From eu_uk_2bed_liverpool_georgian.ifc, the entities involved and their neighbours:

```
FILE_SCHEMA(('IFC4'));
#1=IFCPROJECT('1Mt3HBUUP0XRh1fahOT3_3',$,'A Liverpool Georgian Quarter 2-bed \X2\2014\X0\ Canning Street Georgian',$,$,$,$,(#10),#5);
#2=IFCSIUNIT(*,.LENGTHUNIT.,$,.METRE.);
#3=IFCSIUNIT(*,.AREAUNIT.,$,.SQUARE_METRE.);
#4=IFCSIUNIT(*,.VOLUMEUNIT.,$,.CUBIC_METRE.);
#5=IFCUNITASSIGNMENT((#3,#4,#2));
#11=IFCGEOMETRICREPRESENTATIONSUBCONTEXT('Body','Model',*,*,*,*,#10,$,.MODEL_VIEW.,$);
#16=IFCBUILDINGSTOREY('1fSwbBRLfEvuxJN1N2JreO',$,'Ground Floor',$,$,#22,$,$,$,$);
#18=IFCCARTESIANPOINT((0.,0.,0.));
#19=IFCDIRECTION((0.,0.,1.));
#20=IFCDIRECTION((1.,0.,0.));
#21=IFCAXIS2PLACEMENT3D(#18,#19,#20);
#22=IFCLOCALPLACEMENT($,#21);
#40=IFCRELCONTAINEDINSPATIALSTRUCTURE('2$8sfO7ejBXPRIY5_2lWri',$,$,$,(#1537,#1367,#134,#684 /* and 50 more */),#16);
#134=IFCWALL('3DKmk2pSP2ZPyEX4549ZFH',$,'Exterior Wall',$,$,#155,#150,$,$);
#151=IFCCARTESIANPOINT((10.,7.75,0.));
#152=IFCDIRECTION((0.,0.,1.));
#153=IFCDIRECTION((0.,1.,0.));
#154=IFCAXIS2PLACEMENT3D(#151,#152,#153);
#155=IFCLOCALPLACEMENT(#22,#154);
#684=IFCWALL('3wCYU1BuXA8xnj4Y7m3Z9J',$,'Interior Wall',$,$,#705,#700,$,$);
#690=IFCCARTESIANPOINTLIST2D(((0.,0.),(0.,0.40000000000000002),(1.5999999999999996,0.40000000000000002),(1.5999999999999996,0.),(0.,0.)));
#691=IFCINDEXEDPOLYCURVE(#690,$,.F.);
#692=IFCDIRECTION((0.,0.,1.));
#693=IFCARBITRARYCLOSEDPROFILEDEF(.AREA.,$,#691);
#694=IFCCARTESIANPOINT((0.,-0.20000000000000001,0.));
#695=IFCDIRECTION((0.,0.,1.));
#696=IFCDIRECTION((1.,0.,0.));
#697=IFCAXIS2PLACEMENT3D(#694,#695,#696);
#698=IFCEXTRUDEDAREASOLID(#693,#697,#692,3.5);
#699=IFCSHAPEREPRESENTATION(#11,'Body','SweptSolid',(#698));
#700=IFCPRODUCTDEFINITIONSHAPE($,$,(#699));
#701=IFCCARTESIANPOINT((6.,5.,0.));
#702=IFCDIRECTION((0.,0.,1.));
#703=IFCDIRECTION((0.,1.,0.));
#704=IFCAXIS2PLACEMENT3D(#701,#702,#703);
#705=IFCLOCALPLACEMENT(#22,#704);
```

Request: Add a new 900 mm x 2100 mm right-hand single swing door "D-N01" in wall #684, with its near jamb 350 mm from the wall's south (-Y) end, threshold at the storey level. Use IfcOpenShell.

```python
import numpy as np
import ifcopenshell
import ifcopenshell.api.feature
import ifcopenshell.api.geometry
import ifcopenshell.api.root
import ifcopenshell.api.spatial
import ifcopenshell.geom
import ifcopenshell.util.element
import ifcopenshell.util.placement
import ifcopenshell.util.representation
import ifcopenshell.util.shape
import ifcopenshell.util.unit

model = ifcopenshell.open("eu_uk_2bed_liverpool_georgian.ifc")
unit_scale = ifcopenshell.util.unit.calculate_unit_scale(model)
settings = ifcopenshell.geom.settings()


def volume(element):
    """Net volume in cubic metres, openings subtracted."""
    shape = ifcopenshell.geom.create_shape(settings, element)
    return ifcopenshell.util.shape.get_volume(shape.geometry)


wall = model.by_id(684)
storey = ifcopenshell.util.element.get_container(wall, ifc_class="IfcBuildingStorey")
context = ifcopenshell.util.representation.get_context(model, "Model", "Body", "MODEL_VIEW")
before = volume(wall)

width, height, from_end, sill = 0.9, 2.1, 0.35, 0.0  # metres

# The wall runs along its own X axis, and the end named is its -X end.
wall_shape = ifcopenshell.geom.create_shape(settings, wall)
x, y, z = ifcopenshell.util.shape.get_vertices(wall_shape.geometry).T
start = x.min() + from_end
face, thickness = float(y.min()), float(y.max() - y.min())
wall_matrix = ifcopenshell.util.placement.get_local_placement(wall.ObjectPlacement)
level = ifcopenshell.util.placement.get_local_placement(storey.ObjectPlacement)[2, 3]


def in_wall(x, y):
    """Placement at x, y metres in the wall's axes, at sill height."""
    matrix = wall_matrix.copy()
    matrix[:, 3] = wall_matrix @ np.array([x / unit_scale, y / unit_scale, 0.0, 1.0])
    matrix[2, 3] = level + sill / unit_scale
    return matrix


# Opening: a box that overshoots both wall faces by 50 mm.
opening = ifcopenshell.api.root.create_entity(model, ifc_class="IfcOpeningElement", predefined_type="OPENING")
box = ifcopenshell.api.geometry.add_wall_representation(
    model, context=context, length=width, height=height, thickness=thickness + 0.1
)
ifcopenshell.api.geometry.assign_representation(model, product=opening, representation=box)
ifcopenshell.api.geometry.edit_object_placement(model, product=opening, matrix=in_wall(start, face - 0.05), is_si=False)
ifcopenshell.api.feature.add_feature(model, feature=opening, element=wall)

door = ifcopenshell.api.root.create_entity(model, ifc_class="IfcDoor", name="D-N01", predefined_type="DOOR")
door.OverallWidth, door.OverallHeight = width / unit_scale, height / unit_scale
door.OperationType = "SINGLE_SWING_RIGHT"
body = ifcopenshell.api.geometry.add_door_representation(
    model,
    context=context,
    overall_width=door.OverallWidth,
    overall_height=door.OverallHeight,
    operation_type="SINGLE_SWING_RIGHT",
    lining_properties={"LiningDepth": thickness / unit_scale, "ThresholdDepth": thickness / unit_scale},
)
ifcopenshell.api.geometry.assign_representation(model, product=door, representation=body)
ifcopenshell.api.spatial.assign_container(model, products=[door], relating_structure=storey)
ifcopenshell.api.feature.add_filling(model, opening=opening, element=door)

# The lining spans the wall, so the door starts at the wall face.
ifcopenshell.api.geometry.edit_object_placement(model, product=door, matrix=in_wall(start, face), is_si=False)

after = volume(wall)

print(f"wall volume {before:.3f} -> {after:.3f} m3")

model.write("eu_uk_2bed_liverpool_georgian_rev.ifc")
```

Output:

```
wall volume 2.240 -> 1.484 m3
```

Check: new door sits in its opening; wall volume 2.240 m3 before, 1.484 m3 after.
